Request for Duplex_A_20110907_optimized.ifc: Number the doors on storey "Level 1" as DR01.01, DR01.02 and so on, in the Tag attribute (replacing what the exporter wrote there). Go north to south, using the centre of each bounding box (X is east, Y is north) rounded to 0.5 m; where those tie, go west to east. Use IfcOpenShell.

First a look at what the model holds.

```python
import ifcopenshell
import ifcopenshell.util.element
import ifcopenshell.util.placement

model = ifcopenshell.open("Duplex_A_20110907_optimized.ifc")
print(model.schema)
storey = next(s for s in model.by_type("IfcBuildingStorey") if s.Name == "Level 1")
doors = [e for e in ifcopenshell.util.element.get_decomposition(storey) if e.is_a("IfcDoor")]
for e in sorted(doors, key=lambda e: e.id()):
    origin = ifcopenshell.util.placement.get_local_placement(e.ObjectPlacement)[:3, 3]
    print(e.id(), e.Tag, e.Name, origin.round(2) + 0.0, sep=" | ")
```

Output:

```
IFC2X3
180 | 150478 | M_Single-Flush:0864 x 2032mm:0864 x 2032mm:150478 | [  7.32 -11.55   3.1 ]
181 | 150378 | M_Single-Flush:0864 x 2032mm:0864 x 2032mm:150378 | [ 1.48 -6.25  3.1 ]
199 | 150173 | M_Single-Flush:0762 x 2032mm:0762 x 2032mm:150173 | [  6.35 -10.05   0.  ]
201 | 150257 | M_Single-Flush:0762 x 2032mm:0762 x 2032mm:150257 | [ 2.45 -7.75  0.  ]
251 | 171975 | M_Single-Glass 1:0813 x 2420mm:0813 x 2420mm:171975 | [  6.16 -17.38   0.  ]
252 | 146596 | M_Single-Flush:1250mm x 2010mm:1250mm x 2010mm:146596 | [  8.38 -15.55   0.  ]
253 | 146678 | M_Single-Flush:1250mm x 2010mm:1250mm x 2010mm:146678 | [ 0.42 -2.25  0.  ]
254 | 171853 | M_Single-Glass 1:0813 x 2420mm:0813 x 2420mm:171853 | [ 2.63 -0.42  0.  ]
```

```python
import ifcopenshell
import ifcopenshell.geom
import ifcopenshell.util.element
import ifcopenshell.util.shape

model = ifcopenshell.open("Duplex_A_20110907_optimized.ifc")
settings = ifcopenshell.geom.settings()
settings.set("use-world-coords", True)


def centre(element):
    shape = ifcopenshell.geom.create_shape(settings, element)
    return ifcopenshell.util.shape.get_bbox_centroid(shape.geometry)


storey = next(s for s in model.by_type("IfcBuildingStorey") if s.Name == "Level 1")
doors = [e for e in ifcopenshell.util.element.get_decomposition(storey) if e.is_a("IfcDoor")]

# Insertion points can sit at a corner or the storey origin, so sort by the geometry (in metres).
centres = {e: centre(e) for e in doors}
doors.sort(key=lambda e: (-round(centres[e][1] / 0.5), centres[e][0]))

for i, e in enumerate(doors, start=1):
    number = f"DR01.{i:02d}"
    e.Tag = number
    print(e.id(), number)

model.write("Duplex_A_20110907_optimized-out.ifc")
```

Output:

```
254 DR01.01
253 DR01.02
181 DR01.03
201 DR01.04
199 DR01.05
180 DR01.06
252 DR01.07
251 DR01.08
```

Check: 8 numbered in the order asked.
